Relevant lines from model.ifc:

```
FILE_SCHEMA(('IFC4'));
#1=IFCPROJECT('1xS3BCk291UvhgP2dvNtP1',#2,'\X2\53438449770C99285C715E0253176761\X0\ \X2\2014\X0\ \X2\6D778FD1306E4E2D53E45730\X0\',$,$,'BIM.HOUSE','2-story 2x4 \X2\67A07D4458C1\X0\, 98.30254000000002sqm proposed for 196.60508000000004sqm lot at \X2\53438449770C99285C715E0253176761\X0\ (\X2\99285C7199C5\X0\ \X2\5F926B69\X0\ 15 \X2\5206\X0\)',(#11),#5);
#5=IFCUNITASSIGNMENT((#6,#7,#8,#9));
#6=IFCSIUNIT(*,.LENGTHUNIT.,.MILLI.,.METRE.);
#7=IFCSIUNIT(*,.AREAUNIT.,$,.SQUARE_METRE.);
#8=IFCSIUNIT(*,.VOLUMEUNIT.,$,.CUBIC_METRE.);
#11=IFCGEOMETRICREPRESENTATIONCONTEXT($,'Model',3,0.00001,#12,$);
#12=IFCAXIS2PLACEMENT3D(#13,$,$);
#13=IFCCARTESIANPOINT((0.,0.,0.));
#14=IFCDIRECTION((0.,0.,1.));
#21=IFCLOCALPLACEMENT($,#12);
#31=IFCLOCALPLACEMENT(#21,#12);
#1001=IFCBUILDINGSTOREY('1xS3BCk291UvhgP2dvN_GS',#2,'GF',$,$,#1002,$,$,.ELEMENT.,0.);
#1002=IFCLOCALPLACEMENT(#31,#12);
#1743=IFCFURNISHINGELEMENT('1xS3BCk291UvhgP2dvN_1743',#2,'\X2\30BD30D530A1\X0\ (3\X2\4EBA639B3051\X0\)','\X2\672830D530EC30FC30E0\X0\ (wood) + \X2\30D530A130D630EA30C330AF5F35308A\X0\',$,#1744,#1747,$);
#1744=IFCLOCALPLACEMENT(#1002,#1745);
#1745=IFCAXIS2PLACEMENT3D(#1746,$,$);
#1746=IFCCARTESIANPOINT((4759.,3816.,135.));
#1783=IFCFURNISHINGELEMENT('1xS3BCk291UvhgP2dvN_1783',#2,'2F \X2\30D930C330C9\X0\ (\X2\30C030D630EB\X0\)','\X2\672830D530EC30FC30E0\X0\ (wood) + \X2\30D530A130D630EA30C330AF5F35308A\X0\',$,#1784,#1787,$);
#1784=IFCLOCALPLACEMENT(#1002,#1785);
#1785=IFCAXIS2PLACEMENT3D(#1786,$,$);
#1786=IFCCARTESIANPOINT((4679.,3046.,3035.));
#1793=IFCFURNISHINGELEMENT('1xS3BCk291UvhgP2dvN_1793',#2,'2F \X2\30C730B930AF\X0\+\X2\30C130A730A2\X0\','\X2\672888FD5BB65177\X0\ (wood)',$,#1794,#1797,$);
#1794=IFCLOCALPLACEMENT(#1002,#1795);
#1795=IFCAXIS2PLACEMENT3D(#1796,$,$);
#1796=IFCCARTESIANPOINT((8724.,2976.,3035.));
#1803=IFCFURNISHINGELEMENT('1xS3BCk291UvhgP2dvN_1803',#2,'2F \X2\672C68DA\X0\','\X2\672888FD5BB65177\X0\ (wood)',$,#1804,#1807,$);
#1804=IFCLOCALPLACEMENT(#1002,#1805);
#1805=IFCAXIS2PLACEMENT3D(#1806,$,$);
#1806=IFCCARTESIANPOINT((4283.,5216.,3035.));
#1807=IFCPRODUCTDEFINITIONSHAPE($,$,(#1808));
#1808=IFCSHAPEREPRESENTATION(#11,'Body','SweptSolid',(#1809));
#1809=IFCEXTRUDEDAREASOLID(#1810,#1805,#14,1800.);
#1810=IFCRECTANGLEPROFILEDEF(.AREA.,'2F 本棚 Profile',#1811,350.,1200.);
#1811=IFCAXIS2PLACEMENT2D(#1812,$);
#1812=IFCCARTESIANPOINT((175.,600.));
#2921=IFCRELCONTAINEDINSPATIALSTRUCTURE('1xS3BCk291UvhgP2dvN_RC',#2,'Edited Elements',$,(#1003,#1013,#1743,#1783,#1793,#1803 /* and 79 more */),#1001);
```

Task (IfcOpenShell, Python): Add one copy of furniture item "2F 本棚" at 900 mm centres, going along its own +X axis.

```python
import ifcopenshell
import ifcopenshell.api.geometry
import ifcopenshell.api.root
import ifcopenshell.util.element
import ifcopenshell.util.placement
import ifcopenshell.util.unit

model = ifcopenshell.open("model.ifc")
unit_scale = ifcopenshell.util.unit.calculate_unit_scale(model)


def reuse_history(source, copy):
    """copy_class also copies each property set's owner history, people and application; keep the originals."""
    for rel in copy.IsDefinedBy:
        if rel.is_a("IfcRelDefinesByProperties") and (history := rel.RelatingPropertyDefinition.OwnerHistory):
            rel.RelatingPropertyDefinition.OwnerHistory = source.OwnerHistory
            ifcopenshell.util.element.remove_deep2(model, history)


source = model.by_guid("1xS3BCk291UvhgP2dvN_1803")
base = ifcopenshell.util.placement.get_local_placement(source.ObjectPlacement)
step = base[:3, 0] * 0.9 / unit_scale

for i in range(1, 2):
    copy = ifcopenshell.api.root.copy_class(model, product=source)
    copy.Representation = ifcopenshell.util.element.copy_deep(
        model, source.Representation, exclude=["IfcGeometricRepresentationContext", "IfcRepresentationMap"]
    )
    reuse_history(source, copy)
    matrix = base.copy()
    matrix[:3, 3] += i * step
    print("added at", matrix[:3, 3].round(3) + 0.0)
    ifcopenshell.api.geometry.edit_object_placement(model, product=copy, matrix=matrix, is_si=False)

model.write("model-out.ifc")
```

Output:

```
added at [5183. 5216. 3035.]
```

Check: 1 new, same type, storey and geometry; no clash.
